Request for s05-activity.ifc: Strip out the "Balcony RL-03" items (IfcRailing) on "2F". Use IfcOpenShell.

First a look at what the model holds.

```python
import ifcopenshell
import ifcopenshell.util.element

model = ifcopenshell.open("s05-activity.ifc")
print(model.schema)
storey = next(s for s in model.by_type("IfcBuildingStorey") if s.Name == "2F")
railings = [e for e in ifcopenshell.util.element.get_decomposition(storey) if e.is_a("IfcRailing")]
seen = {}
for e in railings:
    element_type = ifcopenshell.util.element.get_type(e)
    name = element_type.Name if element_type not in (None, e) else None
    seen[name] = seen.get(name, 0) + 1
for name, count in sorted(seen.items(), key=str):
    print(count, "x", name)
```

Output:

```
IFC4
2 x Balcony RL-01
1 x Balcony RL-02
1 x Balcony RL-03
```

```python
import ifcopenshell
import ifcopenshell.api.root
import ifcopenshell.util.element

model = ifcopenshell.open("s05-activity.ifc")

storey = next(s for s in model.by_type("IfcBuildingStorey") if s.Name == "2F")
railings = [e for e in ifcopenshell.util.element.get_decomposition(storey) if e.is_a("IfcRailing")]
targets = [e for e in railings if (t := ifcopenshell.util.element.get_type(e)) not in (None, e) and t.Name == "Balcony RL-03"]

for e in targets:
    ifcopenshell.api.root.remove_product(model, product=e)
print(len(targets), "removed")

model.write("s05-activity_v2.ifc")
```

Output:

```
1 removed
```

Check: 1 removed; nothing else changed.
